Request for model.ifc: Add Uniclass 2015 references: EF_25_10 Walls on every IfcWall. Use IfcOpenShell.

First a look at what the model holds.

```python
import ifcopenshell

model = ifcopenshell.open("model.ifc")
print(model.schema)
print("classifications:", [c.Name for c in model.by_type("IfcClassification")])
for ifc_class in ("IfcDoor", "IfcRoof", "IfcStair", "IfcWall", "IfcWindow"):
    print(ifc_class, len(model.by_type(ifc_class)))
```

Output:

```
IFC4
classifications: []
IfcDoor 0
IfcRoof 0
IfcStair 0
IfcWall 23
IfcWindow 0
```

```python
import ifcopenshell
import ifcopenshell.api.classification

model = ifcopenshell.open("model.ifc")

system = ifcopenshell.api.classification.add_classification(model, classification="Uniclass 2015")

codes = {
    "IfcWall": ("EF_25_10", "Walls"),
}
for ifc_class, (code, name) in codes.items():
    products = model.by_type(ifc_class)
    ifcopenshell.api.classification.add_reference(
        model, products=products, classification=system, identification=code, name=name
    )
    print(code, len(products))

model.write("model_updated.ifc")
```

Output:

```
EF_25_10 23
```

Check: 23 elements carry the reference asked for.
